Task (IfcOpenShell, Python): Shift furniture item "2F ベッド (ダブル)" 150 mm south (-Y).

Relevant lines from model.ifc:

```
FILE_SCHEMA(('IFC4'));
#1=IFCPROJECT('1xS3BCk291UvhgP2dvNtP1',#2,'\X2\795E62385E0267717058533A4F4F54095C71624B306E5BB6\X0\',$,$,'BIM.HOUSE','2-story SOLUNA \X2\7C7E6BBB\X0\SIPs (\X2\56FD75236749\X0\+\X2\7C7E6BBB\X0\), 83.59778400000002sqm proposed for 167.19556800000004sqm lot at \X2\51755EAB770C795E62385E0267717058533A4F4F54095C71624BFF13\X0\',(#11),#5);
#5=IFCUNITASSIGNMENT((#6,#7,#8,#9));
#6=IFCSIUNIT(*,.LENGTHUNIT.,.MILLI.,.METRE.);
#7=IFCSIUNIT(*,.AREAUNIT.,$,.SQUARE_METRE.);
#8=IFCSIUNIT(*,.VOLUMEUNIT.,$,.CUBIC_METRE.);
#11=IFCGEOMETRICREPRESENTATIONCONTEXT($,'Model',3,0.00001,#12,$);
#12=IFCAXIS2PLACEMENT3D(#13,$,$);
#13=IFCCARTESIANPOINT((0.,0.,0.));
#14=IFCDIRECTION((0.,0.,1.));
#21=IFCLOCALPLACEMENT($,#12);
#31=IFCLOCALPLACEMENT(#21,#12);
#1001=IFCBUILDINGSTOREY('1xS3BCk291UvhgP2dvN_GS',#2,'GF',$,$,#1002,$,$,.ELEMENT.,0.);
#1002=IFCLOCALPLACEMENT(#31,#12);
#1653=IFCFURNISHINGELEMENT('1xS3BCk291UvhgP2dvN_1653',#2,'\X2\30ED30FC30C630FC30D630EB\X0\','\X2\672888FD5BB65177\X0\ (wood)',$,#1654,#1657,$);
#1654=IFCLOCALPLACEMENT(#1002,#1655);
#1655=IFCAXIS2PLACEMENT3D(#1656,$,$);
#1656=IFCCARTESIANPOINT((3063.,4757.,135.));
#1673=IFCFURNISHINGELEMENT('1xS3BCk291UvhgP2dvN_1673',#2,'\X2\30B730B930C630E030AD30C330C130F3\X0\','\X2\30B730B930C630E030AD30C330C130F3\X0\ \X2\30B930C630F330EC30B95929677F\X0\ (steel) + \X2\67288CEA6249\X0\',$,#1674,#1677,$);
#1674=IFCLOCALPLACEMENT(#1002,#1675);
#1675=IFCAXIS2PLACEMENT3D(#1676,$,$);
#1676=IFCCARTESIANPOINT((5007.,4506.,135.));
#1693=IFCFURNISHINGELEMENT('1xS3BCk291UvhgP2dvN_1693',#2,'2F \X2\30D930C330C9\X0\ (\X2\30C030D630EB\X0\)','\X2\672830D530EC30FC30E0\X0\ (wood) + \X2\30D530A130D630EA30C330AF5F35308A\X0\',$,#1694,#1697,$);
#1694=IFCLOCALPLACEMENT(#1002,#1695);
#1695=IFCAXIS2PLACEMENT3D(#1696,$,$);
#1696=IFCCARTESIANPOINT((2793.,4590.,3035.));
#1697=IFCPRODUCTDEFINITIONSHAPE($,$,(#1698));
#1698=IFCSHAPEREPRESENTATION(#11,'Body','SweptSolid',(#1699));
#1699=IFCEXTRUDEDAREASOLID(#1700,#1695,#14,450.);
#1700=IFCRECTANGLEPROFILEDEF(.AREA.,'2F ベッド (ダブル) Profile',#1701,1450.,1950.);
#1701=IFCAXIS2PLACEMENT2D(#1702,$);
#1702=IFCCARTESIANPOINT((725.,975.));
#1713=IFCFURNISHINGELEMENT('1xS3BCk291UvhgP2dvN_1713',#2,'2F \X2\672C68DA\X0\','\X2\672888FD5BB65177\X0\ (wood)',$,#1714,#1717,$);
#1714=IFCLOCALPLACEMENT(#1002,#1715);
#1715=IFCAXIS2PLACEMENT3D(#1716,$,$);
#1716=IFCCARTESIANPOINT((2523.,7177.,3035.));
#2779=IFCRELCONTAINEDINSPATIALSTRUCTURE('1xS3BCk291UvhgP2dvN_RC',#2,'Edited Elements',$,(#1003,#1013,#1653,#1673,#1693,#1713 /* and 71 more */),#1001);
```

```python
import ifcopenshell
import ifcopenshell.api.geometry
import ifcopenshell.util.placement

model = ifcopenshell.open("model.ifc")

item = model.by_guid("1xS3BCk291UvhgP2dvN_1693")
matrix = ifcopenshell.util.placement.get_local_placement(item.ObjectPlacement)
matrix[1, 3] -= 150.0
ifcopenshell.api.geometry.edit_object_placement(model, product=item, matrix=matrix, is_si=False)

print(ifcopenshell.util.placement.get_local_placement(item.ObjectPlacement).round(3) + 0.0)

model.write("model_v2.ifc")
```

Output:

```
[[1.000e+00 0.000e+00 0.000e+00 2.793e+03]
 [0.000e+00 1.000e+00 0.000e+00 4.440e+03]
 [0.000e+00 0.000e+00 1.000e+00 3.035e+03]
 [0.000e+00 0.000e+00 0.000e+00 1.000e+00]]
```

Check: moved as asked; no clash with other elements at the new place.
